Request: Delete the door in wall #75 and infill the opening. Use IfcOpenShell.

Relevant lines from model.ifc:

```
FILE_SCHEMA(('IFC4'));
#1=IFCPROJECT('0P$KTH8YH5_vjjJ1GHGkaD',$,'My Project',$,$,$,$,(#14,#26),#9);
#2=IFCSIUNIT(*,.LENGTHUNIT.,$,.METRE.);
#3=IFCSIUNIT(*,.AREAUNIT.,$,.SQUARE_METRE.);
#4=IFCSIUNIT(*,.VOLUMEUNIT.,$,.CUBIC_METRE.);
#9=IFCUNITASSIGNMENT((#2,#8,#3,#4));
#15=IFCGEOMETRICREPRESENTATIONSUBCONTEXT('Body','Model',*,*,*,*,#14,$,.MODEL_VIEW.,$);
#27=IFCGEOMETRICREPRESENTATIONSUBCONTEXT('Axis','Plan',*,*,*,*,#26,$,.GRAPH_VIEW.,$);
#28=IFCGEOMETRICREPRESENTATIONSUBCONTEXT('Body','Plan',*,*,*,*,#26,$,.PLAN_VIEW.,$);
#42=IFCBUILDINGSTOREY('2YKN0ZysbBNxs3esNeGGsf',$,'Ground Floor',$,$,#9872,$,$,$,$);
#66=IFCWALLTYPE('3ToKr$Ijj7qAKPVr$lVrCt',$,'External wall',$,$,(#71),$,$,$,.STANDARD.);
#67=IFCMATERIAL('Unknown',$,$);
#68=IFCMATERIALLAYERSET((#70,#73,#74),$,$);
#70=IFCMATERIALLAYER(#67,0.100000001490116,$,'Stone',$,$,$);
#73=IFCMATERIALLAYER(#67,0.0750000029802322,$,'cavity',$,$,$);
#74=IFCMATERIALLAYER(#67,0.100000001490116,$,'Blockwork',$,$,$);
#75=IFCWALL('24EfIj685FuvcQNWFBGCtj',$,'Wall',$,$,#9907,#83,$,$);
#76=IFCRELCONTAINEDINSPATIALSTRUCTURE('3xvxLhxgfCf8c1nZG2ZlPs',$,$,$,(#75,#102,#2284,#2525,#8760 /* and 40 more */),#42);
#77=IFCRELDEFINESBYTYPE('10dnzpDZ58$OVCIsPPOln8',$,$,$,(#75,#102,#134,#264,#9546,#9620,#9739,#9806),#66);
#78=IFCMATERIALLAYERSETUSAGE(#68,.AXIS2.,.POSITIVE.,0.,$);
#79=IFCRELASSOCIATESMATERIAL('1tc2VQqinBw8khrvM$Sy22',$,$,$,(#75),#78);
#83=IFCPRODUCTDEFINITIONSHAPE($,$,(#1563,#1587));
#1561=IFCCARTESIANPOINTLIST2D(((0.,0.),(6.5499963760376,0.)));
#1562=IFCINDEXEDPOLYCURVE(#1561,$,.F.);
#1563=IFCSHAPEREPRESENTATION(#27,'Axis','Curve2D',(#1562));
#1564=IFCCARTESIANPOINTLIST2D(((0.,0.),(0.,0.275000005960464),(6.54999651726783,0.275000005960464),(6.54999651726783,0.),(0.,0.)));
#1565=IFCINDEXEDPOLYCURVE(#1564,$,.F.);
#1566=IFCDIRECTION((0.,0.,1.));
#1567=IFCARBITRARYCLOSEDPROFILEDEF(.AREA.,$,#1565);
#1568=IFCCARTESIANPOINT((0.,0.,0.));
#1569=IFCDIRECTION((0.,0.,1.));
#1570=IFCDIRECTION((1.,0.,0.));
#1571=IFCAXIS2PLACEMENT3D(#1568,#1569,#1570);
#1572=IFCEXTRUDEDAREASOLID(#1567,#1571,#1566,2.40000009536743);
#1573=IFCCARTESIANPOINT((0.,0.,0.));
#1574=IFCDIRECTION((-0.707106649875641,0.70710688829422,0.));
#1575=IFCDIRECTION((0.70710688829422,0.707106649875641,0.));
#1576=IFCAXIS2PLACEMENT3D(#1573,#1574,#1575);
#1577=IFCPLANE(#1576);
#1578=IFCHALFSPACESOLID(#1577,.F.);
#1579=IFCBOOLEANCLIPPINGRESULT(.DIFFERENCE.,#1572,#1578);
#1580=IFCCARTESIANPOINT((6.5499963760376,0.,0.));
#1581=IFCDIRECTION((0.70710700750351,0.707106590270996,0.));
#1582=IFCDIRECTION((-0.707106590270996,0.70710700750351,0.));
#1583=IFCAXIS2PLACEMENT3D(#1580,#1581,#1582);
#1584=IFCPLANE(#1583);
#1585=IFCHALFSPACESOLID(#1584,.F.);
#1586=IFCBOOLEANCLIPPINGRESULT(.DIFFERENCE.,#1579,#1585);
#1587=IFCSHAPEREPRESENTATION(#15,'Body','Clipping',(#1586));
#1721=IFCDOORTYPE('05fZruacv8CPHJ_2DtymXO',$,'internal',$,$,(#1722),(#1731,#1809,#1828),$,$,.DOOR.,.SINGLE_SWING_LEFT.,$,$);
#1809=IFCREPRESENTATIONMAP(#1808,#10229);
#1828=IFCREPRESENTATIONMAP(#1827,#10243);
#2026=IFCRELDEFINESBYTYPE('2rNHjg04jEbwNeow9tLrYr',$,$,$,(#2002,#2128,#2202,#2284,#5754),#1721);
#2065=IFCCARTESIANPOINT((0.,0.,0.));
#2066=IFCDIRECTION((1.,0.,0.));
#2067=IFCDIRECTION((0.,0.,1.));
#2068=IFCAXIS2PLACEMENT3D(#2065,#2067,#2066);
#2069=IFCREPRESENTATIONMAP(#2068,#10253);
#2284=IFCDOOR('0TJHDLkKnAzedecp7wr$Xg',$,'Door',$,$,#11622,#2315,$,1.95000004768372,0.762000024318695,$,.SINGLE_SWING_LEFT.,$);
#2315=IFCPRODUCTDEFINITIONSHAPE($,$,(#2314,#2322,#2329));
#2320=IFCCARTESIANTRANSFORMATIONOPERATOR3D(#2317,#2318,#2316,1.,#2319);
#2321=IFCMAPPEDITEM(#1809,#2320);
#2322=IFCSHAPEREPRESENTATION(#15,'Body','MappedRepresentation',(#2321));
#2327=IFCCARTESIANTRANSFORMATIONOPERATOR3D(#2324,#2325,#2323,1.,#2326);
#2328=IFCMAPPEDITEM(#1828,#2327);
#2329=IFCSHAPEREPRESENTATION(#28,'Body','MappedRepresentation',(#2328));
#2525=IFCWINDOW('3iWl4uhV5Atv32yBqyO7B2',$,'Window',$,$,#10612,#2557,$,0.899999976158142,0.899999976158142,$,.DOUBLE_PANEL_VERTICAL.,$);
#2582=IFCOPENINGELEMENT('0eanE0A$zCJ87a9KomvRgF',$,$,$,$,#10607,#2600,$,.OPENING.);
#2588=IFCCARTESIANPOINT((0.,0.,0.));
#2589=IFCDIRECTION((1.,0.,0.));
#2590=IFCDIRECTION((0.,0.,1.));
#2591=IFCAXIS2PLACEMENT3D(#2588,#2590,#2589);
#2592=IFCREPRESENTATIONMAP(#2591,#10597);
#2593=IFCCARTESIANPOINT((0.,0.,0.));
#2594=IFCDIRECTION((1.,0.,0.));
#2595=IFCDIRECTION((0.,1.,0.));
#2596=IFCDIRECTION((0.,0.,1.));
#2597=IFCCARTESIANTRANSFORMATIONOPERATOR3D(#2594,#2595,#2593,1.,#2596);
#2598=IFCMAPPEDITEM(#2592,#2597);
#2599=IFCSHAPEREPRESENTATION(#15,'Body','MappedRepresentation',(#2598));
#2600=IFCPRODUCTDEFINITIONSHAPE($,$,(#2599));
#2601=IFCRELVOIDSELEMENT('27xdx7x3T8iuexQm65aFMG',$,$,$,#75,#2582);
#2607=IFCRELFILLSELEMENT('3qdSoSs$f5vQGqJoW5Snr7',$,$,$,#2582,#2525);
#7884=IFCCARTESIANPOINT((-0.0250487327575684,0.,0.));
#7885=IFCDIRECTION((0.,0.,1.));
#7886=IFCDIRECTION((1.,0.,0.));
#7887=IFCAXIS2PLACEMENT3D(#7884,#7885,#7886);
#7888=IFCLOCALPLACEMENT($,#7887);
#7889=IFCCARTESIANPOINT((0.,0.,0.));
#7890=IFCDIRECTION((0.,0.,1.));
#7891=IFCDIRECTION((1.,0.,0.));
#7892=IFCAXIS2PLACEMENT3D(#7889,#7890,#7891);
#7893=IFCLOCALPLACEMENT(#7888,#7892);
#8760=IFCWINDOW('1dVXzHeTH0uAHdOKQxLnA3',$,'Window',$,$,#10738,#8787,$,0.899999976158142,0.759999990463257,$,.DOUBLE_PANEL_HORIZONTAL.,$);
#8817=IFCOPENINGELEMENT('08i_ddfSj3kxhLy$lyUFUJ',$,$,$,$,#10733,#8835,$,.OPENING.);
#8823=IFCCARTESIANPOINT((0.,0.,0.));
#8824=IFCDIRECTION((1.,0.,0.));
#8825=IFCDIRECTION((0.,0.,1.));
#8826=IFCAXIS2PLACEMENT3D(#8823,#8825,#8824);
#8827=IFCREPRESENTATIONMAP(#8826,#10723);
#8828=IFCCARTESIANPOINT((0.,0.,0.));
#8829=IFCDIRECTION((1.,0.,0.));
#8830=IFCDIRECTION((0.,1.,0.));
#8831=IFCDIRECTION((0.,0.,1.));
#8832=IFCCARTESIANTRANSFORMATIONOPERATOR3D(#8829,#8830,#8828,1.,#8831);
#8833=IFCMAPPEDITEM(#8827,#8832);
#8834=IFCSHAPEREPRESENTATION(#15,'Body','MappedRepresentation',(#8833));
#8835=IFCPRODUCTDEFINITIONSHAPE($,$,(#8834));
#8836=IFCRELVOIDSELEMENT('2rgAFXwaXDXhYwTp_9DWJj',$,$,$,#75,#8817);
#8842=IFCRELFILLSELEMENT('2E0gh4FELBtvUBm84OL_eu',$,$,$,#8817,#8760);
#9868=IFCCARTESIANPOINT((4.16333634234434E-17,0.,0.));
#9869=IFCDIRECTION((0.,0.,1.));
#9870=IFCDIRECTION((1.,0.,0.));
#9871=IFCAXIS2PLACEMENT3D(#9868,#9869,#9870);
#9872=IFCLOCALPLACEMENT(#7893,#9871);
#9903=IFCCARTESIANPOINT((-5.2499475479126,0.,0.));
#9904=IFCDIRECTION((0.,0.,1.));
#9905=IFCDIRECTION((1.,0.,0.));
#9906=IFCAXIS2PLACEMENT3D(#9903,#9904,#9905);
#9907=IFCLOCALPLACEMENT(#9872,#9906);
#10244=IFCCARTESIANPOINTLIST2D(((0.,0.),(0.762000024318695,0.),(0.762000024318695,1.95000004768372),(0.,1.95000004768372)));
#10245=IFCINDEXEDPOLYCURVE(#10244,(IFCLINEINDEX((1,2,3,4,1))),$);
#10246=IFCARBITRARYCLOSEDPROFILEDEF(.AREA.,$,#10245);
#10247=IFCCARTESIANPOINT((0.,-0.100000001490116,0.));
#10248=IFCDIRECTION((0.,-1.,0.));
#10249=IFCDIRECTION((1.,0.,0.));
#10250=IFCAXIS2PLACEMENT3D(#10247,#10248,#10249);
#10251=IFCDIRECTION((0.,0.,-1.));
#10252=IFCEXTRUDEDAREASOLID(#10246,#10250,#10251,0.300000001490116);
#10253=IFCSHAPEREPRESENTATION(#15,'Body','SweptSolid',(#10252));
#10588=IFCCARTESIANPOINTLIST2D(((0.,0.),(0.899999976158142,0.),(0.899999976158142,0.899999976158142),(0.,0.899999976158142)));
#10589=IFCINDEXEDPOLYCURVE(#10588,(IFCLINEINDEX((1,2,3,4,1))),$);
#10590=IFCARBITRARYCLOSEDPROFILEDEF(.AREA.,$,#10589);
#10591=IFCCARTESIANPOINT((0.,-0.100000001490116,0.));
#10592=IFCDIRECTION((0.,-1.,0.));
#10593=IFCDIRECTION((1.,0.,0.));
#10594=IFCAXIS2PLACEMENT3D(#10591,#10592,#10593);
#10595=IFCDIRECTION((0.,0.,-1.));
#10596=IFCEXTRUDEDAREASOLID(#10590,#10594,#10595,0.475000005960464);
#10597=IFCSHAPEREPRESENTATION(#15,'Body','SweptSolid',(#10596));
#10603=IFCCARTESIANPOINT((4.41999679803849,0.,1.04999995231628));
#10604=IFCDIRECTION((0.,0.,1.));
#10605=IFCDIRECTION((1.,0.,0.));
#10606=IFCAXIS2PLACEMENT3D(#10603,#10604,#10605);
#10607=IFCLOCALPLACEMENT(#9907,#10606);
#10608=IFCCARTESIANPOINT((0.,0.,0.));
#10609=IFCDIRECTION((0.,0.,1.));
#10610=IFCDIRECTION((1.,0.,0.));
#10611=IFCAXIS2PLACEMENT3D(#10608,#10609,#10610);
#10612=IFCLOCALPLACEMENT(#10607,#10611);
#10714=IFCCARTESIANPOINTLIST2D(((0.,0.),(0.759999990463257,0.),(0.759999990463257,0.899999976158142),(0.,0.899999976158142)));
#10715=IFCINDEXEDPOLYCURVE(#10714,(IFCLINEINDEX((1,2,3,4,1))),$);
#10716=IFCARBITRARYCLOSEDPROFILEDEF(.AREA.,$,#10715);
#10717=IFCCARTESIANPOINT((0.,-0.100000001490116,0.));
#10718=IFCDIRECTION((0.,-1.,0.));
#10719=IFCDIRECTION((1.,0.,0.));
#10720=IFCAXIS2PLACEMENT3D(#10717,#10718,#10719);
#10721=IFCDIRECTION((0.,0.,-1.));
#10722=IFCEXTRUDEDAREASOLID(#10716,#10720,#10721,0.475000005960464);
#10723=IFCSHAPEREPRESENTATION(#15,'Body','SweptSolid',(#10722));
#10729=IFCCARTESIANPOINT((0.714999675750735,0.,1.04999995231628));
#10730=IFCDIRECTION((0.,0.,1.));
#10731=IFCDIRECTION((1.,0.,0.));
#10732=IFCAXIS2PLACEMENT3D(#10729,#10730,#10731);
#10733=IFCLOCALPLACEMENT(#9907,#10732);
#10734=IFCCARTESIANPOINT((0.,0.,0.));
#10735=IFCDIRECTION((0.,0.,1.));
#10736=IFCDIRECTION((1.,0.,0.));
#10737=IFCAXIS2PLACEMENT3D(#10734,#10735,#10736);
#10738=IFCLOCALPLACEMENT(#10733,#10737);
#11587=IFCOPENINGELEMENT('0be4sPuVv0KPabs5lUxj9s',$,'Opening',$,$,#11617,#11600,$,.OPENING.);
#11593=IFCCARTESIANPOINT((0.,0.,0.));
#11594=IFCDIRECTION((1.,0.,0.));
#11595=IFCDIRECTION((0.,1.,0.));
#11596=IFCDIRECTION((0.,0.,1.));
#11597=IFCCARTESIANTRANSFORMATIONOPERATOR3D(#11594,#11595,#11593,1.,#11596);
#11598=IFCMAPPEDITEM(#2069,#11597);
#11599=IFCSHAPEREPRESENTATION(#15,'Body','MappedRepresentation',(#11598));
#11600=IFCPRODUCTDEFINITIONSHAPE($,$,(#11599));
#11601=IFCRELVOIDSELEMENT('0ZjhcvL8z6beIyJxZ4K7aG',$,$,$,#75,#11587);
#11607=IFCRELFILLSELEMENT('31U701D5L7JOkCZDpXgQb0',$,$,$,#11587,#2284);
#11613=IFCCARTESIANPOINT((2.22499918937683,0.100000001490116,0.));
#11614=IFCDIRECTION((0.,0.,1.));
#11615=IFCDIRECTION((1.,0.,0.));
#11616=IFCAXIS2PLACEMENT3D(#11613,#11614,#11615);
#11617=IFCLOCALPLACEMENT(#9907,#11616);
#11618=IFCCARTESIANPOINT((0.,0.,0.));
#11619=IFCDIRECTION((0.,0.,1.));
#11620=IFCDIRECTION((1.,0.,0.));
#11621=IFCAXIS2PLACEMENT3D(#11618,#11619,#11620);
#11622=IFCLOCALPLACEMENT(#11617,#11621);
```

```python
import ifcopenshell
import ifcopenshell.api.feature
import ifcopenshell.api.root
import ifcopenshell.geom
import ifcopenshell.util.shape

model = ifcopenshell.open("model.ifc")
settings = ifcopenshell.geom.settings()


def volume(element):
    """Net volume in cubic metres, openings subtracted."""
    shape = ifcopenshell.geom.create_shape(settings, element)
    return ifcopenshell.util.shape.get_volume(shape.geometry)


door = model.by_guid("0TJHDLkKnAzedecp7wr$Xg")
opening = door.FillsVoids[0].RelatingOpeningElement
wall = opening.VoidsElements[0].RelatingBuildingElement
before = volume(wall)

ifcopenshell.api.root.remove_product(model, product=door)
ifcopenshell.api.feature.remove_feature(model, feature=opening)

after = volume(wall)

print(f"wall volume {before:.3f} -> {after:.3f} m3")

model.write("model-out.ifc")
```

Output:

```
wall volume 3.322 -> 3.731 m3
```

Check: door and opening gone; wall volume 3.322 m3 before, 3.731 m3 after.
